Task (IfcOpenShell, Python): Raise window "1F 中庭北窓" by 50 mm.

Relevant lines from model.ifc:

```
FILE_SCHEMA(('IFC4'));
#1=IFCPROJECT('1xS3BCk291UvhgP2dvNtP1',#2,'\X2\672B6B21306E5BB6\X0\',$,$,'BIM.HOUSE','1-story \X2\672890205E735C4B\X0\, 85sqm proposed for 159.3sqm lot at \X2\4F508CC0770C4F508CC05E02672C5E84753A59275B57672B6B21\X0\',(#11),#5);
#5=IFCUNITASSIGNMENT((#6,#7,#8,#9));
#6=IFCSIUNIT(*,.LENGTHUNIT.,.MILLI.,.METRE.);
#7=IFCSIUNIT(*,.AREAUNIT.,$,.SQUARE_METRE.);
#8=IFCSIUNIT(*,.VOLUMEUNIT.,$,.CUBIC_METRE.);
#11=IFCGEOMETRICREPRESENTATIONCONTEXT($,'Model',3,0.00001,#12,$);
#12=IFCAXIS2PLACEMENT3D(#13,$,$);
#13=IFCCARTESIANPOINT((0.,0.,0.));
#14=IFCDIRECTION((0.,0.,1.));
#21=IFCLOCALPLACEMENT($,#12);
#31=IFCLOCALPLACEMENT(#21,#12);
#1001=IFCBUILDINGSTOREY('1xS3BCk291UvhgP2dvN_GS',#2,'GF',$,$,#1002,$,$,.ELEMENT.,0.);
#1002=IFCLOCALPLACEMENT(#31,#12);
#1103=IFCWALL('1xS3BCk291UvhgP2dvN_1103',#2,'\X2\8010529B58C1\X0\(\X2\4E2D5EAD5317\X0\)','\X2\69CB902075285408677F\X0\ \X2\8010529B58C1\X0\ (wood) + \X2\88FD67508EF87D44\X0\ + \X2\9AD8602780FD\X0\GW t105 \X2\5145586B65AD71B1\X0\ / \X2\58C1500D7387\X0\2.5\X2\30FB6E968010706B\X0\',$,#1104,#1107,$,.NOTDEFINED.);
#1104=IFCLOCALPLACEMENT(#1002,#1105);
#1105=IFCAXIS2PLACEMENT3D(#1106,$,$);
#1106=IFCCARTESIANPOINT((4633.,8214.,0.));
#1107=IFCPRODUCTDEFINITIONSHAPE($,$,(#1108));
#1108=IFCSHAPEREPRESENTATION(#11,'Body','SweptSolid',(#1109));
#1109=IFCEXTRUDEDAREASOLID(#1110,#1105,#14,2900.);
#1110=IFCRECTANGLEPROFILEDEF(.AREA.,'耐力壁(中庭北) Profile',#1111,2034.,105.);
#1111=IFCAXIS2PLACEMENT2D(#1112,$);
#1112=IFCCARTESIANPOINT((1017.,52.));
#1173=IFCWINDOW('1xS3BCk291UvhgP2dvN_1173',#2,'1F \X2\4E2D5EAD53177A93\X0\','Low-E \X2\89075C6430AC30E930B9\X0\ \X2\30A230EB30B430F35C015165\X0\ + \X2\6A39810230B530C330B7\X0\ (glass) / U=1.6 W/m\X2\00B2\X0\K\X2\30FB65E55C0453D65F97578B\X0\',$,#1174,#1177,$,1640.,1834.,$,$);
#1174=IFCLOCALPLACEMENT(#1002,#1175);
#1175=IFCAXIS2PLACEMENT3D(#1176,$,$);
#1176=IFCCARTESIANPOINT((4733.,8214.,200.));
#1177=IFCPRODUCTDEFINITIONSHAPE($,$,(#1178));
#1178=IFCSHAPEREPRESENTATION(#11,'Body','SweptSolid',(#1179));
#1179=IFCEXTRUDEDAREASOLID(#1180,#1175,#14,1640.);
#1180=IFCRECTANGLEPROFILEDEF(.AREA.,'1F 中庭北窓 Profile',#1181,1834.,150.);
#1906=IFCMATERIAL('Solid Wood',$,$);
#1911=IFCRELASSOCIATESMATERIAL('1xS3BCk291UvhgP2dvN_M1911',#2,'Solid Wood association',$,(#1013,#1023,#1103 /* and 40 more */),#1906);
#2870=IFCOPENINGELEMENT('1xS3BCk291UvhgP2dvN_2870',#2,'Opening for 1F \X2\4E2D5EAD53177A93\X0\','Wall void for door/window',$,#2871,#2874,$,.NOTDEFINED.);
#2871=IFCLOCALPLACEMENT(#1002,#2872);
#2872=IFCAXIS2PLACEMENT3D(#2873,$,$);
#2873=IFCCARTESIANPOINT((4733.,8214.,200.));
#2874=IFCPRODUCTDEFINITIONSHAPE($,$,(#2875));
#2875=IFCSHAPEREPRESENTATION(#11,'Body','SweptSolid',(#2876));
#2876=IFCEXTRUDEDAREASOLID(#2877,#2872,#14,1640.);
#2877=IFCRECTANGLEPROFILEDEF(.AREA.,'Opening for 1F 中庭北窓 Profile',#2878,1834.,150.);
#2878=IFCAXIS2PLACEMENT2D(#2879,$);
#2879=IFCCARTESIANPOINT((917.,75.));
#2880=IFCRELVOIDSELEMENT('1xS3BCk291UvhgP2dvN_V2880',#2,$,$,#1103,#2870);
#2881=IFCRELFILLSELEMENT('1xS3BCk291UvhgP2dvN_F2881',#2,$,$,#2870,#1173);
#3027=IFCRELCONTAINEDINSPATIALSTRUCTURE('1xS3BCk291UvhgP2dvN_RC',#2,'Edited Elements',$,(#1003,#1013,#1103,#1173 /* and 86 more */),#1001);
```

```python
import numpy as np
import ifcopenshell
import ifcopenshell.api.geometry
import ifcopenshell.util.placement
import ifcopenshell.util.unit

model = ifcopenshell.open("model.ifc")
unit_scale = ifcopenshell.util.unit.calculate_unit_scale(model)

window = model.by_guid("1xS3BCk291UvhgP2dvN_1173")
opening = window.FillsVoids[0].RelatingOpeningElement
dz = 50.0

shift = np.array([0.0, 0.0, dz])
# The window is not placed relative to its opening, so move both.
for product in (opening, window):
    matrix = ifcopenshell.util.placement.get_local_placement(product.ObjectPlacement)
    matrix[:3, 3] += shift
    ifcopenshell.api.geometry.edit_object_placement(model, product=product, matrix=matrix, is_si=False)

print(f"moved by {dz * unit_scale:+.3f} m")

model.write("model_v2.ifc")
```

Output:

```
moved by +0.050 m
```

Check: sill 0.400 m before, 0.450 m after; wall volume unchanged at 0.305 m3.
